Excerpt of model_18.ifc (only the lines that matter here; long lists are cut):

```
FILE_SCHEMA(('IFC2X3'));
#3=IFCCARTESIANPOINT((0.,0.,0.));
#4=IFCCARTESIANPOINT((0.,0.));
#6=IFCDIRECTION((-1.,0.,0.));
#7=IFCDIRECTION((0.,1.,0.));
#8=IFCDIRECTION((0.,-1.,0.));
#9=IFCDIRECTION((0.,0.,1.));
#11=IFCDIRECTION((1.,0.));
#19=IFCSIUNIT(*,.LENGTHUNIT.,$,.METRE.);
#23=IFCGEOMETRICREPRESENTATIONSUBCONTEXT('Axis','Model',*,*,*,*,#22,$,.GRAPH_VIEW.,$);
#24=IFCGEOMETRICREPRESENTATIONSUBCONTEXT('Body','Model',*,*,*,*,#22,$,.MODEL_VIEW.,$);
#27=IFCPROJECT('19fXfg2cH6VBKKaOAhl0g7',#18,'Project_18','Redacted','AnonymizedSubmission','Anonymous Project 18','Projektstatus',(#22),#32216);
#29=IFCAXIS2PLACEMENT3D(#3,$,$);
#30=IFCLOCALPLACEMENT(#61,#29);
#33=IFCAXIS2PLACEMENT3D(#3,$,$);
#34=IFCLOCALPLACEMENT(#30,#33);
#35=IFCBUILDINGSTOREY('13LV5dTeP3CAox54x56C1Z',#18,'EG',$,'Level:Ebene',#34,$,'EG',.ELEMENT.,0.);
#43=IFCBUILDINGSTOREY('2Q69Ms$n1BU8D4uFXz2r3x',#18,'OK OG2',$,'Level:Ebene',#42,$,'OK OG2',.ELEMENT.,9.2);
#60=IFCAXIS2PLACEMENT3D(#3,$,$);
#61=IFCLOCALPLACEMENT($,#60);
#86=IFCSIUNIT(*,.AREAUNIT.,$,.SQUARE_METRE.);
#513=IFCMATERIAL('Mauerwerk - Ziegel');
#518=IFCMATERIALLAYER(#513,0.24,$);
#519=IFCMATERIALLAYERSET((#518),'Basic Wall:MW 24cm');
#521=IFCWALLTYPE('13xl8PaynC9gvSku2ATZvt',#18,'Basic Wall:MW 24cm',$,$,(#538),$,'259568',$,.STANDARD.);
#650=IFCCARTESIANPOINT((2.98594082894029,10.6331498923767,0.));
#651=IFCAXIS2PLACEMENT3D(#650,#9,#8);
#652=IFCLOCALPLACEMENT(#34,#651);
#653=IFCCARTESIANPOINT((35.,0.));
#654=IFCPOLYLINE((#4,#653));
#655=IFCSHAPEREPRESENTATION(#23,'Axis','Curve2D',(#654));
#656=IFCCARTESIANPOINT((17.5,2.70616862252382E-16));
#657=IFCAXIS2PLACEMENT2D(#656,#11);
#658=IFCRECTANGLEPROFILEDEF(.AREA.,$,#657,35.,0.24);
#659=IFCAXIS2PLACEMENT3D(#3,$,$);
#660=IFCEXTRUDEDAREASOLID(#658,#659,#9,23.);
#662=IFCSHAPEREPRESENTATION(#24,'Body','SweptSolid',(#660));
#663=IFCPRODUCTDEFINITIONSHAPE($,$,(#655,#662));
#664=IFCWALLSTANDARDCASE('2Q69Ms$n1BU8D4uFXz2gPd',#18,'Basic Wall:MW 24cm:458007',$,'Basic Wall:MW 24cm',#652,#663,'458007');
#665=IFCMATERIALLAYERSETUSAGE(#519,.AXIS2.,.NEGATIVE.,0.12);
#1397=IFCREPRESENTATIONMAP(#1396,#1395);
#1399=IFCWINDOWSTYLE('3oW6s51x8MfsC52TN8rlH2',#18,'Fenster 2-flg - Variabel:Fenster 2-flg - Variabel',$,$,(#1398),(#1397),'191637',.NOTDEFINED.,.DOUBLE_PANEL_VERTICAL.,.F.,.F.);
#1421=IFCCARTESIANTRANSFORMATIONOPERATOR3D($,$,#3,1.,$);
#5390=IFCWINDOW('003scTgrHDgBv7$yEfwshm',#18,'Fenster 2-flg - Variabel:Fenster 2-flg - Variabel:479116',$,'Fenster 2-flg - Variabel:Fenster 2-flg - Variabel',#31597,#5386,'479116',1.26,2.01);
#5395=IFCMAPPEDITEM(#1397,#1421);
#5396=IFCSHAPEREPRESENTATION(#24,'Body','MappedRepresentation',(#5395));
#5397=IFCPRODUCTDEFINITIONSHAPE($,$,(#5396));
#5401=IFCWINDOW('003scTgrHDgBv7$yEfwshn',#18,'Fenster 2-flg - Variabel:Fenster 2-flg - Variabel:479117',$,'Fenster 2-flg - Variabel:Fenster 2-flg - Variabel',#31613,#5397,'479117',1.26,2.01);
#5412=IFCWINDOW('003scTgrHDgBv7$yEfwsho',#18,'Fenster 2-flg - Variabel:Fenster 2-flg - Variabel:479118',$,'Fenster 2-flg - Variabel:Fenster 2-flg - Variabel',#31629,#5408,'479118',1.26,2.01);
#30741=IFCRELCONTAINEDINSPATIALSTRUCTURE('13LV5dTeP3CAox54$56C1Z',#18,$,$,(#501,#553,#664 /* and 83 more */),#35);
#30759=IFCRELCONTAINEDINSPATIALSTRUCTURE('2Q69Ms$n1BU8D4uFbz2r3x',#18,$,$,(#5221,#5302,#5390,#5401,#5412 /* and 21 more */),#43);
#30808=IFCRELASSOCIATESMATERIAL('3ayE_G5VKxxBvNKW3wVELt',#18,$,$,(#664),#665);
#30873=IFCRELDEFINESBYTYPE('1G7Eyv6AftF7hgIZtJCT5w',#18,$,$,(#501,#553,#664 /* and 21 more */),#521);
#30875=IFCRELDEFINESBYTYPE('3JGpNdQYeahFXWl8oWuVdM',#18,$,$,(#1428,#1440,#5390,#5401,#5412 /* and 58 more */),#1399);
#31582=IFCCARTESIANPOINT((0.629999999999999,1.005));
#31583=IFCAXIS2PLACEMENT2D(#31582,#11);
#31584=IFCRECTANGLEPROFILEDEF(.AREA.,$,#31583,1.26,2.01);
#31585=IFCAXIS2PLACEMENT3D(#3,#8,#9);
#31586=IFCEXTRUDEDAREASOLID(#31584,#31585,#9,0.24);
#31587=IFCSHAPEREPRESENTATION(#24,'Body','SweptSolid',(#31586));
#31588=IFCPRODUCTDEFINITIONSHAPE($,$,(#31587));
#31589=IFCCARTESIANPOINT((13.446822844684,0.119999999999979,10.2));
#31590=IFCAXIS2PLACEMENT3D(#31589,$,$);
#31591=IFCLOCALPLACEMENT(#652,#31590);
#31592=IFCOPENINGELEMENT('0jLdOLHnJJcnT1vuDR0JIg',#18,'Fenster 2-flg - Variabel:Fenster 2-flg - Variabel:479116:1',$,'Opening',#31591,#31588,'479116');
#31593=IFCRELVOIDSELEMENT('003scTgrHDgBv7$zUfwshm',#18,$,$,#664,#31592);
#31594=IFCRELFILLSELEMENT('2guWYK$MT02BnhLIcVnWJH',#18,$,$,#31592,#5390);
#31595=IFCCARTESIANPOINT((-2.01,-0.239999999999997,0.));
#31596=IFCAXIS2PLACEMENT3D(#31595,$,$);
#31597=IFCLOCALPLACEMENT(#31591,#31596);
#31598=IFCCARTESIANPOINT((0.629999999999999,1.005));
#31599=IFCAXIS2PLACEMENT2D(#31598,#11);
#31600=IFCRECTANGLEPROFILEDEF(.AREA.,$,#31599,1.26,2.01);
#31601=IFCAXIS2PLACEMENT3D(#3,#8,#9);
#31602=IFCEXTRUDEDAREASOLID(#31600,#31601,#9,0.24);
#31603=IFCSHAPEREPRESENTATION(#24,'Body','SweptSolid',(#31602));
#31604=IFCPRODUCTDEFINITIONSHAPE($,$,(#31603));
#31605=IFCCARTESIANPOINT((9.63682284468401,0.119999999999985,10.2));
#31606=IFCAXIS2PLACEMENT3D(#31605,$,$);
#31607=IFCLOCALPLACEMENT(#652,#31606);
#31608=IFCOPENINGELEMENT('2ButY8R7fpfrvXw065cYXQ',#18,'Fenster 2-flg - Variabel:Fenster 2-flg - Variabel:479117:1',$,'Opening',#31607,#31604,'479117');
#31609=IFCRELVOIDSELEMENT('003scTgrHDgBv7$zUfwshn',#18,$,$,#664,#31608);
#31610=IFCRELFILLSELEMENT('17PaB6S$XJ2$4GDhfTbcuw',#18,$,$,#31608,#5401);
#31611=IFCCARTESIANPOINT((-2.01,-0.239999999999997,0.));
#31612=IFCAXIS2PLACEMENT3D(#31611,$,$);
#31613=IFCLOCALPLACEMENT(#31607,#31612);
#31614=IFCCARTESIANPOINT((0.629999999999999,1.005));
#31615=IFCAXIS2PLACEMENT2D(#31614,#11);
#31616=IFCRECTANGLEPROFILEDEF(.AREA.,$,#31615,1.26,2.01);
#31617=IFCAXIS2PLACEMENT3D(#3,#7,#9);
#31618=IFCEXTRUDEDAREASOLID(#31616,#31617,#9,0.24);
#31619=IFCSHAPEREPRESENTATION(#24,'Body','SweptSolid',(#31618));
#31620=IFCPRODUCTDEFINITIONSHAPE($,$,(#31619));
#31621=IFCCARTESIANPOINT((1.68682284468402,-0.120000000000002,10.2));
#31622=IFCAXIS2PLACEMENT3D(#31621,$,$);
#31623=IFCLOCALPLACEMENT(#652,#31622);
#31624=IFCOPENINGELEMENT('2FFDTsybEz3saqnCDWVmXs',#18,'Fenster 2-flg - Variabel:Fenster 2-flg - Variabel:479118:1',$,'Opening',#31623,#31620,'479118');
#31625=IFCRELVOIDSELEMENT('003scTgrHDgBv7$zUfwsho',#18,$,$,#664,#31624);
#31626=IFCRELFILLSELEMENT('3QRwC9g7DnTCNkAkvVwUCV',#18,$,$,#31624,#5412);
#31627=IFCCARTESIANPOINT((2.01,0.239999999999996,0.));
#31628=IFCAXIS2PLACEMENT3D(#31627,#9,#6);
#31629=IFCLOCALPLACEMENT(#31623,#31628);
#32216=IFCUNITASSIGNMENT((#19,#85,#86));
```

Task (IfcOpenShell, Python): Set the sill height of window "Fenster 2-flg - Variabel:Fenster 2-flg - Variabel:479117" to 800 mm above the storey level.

```python
import numpy as np
import ifcopenshell
import ifcopenshell.api.geometry
import ifcopenshell.geom
import ifcopenshell.util.element
import ifcopenshell.util.placement
import ifcopenshell.util.shape
import ifcopenshell.util.unit

model = ifcopenshell.open("model_18.ifc")
unit_scale = ifcopenshell.util.unit.calculate_unit_scale(model)

window = model.by_guid("003scTgrHDgBv7$yEfwshn")
opening = window.FillsVoids[0].RelatingOpeningElement
storey = ifcopenshell.util.element.get_container(window, ifc_class="IfcBuildingStorey")
level = ifcopenshell.util.placement.get_local_placement(storey.ObjectPlacement)[2, 3]

# The opening's origin need not be at the sill, so measure its lowest point.
shape = ifcopenshell.geom.create_shape(ifcopenshell.geom.settings(), opening)
bottom = ifcopenshell.util.shape.get_shape_bottom_elevation(shape, shape.geometry) / unit_scale
dz = level + 0.8 / unit_scale - bottom

shift = np.array([0.0, 0.0, dz])
# The window is placed relative to its opening, so it follows when the opening moves.
matrix = ifcopenshell.util.placement.get_local_placement(opening.ObjectPlacement)
matrix[:3, 3] += shift
ifcopenshell.api.geometry.edit_object_placement(
    model, product=opening, matrix=matrix, is_si=False, should_transform_children=True
)

print(f"moved by {dz * unit_scale:+.3f} m")

model.write("model_18_updated.ifc")
```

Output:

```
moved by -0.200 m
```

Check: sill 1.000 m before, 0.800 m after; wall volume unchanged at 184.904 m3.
